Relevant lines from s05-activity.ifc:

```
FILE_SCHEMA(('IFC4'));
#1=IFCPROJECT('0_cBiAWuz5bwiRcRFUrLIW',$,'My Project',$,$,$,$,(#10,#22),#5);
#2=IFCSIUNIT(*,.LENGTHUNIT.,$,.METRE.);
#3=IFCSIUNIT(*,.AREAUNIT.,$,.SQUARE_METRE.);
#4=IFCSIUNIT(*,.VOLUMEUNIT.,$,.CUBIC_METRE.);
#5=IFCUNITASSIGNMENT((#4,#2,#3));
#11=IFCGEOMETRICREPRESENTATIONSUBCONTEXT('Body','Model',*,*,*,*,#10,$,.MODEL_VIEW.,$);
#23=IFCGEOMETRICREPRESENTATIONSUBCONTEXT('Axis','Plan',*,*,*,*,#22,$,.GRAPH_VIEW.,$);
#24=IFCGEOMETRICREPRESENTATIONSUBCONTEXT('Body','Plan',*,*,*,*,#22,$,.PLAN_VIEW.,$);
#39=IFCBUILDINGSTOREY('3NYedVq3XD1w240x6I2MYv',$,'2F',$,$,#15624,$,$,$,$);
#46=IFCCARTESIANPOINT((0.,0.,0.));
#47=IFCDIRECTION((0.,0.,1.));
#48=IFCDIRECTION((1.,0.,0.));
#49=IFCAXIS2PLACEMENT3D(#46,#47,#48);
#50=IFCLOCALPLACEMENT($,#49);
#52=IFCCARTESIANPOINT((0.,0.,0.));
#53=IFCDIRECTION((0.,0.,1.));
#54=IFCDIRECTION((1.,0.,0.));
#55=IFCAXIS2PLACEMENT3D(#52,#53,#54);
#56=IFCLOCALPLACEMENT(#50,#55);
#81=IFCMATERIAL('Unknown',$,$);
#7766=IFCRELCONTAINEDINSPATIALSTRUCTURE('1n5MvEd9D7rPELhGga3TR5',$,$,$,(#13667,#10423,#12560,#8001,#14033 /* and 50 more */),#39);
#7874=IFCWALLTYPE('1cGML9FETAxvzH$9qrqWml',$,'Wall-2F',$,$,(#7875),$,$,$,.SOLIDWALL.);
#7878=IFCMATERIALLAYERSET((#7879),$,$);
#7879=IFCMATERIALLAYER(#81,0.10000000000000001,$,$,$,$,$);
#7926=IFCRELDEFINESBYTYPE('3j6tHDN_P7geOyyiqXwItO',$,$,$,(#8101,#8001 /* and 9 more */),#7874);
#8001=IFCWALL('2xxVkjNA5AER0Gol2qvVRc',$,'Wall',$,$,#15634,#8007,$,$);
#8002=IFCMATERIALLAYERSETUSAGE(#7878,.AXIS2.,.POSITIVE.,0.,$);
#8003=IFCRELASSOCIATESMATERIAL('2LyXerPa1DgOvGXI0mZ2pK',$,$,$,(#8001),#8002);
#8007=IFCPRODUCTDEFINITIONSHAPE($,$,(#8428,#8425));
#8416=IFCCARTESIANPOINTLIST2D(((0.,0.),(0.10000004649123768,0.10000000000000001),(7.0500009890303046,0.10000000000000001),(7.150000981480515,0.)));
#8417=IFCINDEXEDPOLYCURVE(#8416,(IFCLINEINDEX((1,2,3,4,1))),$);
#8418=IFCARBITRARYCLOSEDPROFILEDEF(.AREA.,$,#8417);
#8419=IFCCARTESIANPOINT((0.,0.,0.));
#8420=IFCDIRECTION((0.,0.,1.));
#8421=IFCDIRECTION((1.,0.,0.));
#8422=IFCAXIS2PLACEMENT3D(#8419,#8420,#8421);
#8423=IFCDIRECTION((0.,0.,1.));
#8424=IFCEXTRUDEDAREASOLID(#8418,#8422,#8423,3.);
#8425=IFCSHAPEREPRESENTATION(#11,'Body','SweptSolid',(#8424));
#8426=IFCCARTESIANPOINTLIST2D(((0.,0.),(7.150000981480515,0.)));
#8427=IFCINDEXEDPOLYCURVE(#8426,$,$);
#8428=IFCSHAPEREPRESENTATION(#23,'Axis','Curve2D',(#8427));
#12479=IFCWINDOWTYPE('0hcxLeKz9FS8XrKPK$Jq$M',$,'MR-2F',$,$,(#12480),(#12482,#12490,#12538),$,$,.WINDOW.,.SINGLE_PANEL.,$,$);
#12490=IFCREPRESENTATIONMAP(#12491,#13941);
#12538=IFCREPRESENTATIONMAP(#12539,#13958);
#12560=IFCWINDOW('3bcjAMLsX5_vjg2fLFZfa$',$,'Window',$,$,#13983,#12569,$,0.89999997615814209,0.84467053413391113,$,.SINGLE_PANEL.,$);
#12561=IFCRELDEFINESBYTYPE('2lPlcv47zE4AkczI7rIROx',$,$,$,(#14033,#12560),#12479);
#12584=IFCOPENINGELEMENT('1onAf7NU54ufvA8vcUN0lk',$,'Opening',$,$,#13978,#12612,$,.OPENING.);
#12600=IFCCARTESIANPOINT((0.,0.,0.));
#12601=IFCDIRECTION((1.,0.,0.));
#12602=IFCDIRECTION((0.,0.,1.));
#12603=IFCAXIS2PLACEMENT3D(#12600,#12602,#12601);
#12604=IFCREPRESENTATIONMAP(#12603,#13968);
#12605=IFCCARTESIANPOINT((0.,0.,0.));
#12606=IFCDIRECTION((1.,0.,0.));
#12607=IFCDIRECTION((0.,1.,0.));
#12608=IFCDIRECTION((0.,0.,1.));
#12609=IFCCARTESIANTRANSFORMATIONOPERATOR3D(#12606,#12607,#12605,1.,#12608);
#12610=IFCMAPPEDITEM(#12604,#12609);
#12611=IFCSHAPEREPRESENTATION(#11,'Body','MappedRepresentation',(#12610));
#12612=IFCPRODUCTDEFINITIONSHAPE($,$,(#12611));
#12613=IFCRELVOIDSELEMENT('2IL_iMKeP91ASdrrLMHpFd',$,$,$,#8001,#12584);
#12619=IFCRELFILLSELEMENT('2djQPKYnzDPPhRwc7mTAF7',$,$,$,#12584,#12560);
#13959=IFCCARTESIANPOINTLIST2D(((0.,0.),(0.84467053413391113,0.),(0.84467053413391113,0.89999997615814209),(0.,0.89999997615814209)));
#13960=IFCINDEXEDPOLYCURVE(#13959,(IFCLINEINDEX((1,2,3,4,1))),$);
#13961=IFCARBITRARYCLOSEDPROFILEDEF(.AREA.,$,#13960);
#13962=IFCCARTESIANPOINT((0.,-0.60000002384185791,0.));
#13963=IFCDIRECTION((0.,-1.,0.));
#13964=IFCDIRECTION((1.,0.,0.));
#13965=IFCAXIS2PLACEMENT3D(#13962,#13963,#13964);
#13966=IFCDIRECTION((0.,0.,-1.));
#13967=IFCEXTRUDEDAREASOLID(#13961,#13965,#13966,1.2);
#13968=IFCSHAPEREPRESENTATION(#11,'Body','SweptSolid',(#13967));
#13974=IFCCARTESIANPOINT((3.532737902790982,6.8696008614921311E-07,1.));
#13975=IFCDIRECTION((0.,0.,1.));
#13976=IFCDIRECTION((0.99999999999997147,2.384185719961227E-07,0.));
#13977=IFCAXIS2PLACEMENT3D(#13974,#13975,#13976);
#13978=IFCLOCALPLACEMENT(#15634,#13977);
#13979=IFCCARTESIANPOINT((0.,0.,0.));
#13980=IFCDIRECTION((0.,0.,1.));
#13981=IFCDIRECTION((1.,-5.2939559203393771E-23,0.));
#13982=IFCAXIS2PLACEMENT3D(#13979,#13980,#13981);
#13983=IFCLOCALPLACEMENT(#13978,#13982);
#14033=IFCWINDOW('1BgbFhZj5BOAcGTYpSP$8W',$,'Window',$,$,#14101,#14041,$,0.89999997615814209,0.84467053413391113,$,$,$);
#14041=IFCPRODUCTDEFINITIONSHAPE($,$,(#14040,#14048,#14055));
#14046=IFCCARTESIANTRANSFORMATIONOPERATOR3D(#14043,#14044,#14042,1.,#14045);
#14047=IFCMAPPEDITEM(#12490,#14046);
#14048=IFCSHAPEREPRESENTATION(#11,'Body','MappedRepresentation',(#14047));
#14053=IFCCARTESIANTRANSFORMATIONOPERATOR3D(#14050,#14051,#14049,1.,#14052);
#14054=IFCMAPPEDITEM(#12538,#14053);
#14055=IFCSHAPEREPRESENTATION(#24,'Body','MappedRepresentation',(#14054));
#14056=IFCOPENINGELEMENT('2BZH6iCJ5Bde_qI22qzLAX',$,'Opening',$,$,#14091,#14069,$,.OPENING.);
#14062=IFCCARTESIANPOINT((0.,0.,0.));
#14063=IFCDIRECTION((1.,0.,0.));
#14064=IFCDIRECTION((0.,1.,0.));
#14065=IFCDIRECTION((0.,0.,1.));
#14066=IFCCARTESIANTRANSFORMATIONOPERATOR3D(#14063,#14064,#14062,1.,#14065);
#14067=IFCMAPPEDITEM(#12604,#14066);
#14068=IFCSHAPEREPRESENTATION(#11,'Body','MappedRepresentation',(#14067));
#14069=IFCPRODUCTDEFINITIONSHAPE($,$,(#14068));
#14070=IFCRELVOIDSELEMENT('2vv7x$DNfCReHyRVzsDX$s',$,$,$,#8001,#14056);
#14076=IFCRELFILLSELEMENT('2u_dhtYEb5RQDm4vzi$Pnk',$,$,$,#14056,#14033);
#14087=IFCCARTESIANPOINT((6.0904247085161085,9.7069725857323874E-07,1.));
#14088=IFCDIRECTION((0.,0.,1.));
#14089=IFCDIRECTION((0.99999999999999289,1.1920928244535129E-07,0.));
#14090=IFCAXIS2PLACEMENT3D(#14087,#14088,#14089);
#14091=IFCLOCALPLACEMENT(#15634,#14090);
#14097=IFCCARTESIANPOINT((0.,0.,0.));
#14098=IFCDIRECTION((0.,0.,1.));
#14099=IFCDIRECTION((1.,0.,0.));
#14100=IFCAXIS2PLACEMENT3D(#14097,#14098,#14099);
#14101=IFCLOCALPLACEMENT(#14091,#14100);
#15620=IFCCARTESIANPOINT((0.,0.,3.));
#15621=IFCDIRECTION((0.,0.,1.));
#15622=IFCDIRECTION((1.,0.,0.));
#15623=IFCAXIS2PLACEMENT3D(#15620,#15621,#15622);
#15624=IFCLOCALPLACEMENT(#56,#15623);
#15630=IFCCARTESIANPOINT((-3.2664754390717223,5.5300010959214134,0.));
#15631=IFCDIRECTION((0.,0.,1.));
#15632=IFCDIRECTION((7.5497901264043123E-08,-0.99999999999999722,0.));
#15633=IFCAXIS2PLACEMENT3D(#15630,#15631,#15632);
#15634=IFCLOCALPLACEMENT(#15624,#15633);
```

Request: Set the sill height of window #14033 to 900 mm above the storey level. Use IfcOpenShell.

```python
import numpy as np
import ifcopenshell
import ifcopenshell.api.geometry
import ifcopenshell.geom
import ifcopenshell.util.element
import ifcopenshell.util.placement
import ifcopenshell.util.shape
import ifcopenshell.util.unit

model = ifcopenshell.open("s05-activity.ifc")
unit_scale = ifcopenshell.util.unit.calculate_unit_scale(model)

window = model.by_guid("1BgbFhZj5BOAcGTYpSP$8W")
opening = window.FillsVoids[0].RelatingOpeningElement
storey = ifcopenshell.util.element.get_container(window, ifc_class="IfcBuildingStorey")
level = ifcopenshell.util.placement.get_local_placement(storey.ObjectPlacement)[2, 3]

# The opening's origin need not be at the sill, so measure its lowest point.
shape = ifcopenshell.geom.create_shape(ifcopenshell.geom.settings(), opening)
bottom = ifcopenshell.util.shape.get_shape_bottom_elevation(shape, shape.geometry) / unit_scale
dz = level + 0.9 - bottom

shift = np.array([0.0, 0.0, dz])
# The window is placed relative to its opening, so it follows when the opening moves.
matrix = ifcopenshell.util.placement.get_local_placement(opening.ObjectPlacement)
matrix[:3, 3] += shift
ifcopenshell.api.geometry.edit_object_placement(
    model, product=opening, matrix=matrix, is_si=False, should_transform_children=True
)

print(f"moved by {dz * unit_scale:+.3f} m")

model.write("s05-activity_edited.ifc")
```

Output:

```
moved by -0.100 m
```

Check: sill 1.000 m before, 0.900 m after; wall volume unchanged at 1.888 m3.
